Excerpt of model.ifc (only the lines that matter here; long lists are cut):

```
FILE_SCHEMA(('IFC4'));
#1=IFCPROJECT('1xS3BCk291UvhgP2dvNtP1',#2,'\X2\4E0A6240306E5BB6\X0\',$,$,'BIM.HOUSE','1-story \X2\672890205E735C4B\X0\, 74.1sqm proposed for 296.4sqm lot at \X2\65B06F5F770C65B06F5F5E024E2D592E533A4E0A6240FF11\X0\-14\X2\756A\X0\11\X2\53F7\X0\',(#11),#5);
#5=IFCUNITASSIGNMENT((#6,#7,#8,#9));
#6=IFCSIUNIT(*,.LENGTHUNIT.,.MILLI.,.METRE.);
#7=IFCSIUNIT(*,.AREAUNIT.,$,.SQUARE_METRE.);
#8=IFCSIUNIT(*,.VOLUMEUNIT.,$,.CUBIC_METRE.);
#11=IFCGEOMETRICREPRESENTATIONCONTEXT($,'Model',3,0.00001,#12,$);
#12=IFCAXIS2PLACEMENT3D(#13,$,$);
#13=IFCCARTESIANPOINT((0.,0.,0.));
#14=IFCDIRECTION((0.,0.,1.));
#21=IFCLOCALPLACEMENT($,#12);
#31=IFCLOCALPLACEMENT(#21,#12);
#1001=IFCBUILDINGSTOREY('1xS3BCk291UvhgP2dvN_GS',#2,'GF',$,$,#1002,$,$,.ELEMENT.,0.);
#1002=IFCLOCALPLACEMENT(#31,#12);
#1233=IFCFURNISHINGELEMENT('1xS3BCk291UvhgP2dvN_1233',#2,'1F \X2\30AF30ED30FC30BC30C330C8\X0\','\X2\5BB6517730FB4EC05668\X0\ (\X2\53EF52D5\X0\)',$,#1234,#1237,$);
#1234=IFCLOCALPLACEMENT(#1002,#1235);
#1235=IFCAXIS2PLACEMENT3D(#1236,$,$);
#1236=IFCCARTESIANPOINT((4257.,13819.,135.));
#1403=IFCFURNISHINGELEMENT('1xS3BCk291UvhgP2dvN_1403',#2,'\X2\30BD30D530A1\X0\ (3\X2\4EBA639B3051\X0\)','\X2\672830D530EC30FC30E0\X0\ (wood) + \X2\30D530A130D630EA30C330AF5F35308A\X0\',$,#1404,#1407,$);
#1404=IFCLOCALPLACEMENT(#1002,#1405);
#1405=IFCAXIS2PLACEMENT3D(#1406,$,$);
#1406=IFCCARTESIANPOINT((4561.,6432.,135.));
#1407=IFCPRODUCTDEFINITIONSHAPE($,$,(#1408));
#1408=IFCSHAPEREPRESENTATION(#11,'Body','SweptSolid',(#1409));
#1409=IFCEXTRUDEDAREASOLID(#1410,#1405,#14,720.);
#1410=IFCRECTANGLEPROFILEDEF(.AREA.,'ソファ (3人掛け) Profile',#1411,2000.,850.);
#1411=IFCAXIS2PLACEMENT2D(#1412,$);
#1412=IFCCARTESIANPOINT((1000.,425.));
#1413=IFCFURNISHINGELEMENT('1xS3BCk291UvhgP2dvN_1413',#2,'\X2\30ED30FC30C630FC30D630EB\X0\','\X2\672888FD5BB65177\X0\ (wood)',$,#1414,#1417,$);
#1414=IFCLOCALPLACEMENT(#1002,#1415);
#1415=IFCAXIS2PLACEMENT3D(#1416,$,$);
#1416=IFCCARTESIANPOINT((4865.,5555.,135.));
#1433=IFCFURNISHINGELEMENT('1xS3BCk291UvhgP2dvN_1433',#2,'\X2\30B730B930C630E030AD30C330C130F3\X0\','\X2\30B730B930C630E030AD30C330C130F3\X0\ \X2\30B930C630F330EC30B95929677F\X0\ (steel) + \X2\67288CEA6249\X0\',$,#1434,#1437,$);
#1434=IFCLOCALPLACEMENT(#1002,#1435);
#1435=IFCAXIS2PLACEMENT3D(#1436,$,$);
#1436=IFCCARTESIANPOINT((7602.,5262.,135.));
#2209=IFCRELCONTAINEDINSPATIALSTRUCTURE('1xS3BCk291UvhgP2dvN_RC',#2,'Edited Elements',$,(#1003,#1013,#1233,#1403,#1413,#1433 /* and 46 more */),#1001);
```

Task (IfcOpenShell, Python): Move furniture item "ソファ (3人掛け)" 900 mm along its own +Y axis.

```python
import ifcopenshell
import ifcopenshell.api.geometry
import ifcopenshell.util.placement

model = ifcopenshell.open("model.ifc")

item = model.by_id(1403)
matrix = ifcopenshell.util.placement.get_local_placement(item.ObjectPlacement)
matrix[:3, 3] += matrix[:3, 1] * 900.0
ifcopenshell.api.geometry.edit_object_placement(model, product=item, matrix=matrix, is_si=False)

print(ifcopenshell.util.placement.get_local_placement(item.ObjectPlacement).round(3) + 0.0)

model.write("model_v2.ifc")
```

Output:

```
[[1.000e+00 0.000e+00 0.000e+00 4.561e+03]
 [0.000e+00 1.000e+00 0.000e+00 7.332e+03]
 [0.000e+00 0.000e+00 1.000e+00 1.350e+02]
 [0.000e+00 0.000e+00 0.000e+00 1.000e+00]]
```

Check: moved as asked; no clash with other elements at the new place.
